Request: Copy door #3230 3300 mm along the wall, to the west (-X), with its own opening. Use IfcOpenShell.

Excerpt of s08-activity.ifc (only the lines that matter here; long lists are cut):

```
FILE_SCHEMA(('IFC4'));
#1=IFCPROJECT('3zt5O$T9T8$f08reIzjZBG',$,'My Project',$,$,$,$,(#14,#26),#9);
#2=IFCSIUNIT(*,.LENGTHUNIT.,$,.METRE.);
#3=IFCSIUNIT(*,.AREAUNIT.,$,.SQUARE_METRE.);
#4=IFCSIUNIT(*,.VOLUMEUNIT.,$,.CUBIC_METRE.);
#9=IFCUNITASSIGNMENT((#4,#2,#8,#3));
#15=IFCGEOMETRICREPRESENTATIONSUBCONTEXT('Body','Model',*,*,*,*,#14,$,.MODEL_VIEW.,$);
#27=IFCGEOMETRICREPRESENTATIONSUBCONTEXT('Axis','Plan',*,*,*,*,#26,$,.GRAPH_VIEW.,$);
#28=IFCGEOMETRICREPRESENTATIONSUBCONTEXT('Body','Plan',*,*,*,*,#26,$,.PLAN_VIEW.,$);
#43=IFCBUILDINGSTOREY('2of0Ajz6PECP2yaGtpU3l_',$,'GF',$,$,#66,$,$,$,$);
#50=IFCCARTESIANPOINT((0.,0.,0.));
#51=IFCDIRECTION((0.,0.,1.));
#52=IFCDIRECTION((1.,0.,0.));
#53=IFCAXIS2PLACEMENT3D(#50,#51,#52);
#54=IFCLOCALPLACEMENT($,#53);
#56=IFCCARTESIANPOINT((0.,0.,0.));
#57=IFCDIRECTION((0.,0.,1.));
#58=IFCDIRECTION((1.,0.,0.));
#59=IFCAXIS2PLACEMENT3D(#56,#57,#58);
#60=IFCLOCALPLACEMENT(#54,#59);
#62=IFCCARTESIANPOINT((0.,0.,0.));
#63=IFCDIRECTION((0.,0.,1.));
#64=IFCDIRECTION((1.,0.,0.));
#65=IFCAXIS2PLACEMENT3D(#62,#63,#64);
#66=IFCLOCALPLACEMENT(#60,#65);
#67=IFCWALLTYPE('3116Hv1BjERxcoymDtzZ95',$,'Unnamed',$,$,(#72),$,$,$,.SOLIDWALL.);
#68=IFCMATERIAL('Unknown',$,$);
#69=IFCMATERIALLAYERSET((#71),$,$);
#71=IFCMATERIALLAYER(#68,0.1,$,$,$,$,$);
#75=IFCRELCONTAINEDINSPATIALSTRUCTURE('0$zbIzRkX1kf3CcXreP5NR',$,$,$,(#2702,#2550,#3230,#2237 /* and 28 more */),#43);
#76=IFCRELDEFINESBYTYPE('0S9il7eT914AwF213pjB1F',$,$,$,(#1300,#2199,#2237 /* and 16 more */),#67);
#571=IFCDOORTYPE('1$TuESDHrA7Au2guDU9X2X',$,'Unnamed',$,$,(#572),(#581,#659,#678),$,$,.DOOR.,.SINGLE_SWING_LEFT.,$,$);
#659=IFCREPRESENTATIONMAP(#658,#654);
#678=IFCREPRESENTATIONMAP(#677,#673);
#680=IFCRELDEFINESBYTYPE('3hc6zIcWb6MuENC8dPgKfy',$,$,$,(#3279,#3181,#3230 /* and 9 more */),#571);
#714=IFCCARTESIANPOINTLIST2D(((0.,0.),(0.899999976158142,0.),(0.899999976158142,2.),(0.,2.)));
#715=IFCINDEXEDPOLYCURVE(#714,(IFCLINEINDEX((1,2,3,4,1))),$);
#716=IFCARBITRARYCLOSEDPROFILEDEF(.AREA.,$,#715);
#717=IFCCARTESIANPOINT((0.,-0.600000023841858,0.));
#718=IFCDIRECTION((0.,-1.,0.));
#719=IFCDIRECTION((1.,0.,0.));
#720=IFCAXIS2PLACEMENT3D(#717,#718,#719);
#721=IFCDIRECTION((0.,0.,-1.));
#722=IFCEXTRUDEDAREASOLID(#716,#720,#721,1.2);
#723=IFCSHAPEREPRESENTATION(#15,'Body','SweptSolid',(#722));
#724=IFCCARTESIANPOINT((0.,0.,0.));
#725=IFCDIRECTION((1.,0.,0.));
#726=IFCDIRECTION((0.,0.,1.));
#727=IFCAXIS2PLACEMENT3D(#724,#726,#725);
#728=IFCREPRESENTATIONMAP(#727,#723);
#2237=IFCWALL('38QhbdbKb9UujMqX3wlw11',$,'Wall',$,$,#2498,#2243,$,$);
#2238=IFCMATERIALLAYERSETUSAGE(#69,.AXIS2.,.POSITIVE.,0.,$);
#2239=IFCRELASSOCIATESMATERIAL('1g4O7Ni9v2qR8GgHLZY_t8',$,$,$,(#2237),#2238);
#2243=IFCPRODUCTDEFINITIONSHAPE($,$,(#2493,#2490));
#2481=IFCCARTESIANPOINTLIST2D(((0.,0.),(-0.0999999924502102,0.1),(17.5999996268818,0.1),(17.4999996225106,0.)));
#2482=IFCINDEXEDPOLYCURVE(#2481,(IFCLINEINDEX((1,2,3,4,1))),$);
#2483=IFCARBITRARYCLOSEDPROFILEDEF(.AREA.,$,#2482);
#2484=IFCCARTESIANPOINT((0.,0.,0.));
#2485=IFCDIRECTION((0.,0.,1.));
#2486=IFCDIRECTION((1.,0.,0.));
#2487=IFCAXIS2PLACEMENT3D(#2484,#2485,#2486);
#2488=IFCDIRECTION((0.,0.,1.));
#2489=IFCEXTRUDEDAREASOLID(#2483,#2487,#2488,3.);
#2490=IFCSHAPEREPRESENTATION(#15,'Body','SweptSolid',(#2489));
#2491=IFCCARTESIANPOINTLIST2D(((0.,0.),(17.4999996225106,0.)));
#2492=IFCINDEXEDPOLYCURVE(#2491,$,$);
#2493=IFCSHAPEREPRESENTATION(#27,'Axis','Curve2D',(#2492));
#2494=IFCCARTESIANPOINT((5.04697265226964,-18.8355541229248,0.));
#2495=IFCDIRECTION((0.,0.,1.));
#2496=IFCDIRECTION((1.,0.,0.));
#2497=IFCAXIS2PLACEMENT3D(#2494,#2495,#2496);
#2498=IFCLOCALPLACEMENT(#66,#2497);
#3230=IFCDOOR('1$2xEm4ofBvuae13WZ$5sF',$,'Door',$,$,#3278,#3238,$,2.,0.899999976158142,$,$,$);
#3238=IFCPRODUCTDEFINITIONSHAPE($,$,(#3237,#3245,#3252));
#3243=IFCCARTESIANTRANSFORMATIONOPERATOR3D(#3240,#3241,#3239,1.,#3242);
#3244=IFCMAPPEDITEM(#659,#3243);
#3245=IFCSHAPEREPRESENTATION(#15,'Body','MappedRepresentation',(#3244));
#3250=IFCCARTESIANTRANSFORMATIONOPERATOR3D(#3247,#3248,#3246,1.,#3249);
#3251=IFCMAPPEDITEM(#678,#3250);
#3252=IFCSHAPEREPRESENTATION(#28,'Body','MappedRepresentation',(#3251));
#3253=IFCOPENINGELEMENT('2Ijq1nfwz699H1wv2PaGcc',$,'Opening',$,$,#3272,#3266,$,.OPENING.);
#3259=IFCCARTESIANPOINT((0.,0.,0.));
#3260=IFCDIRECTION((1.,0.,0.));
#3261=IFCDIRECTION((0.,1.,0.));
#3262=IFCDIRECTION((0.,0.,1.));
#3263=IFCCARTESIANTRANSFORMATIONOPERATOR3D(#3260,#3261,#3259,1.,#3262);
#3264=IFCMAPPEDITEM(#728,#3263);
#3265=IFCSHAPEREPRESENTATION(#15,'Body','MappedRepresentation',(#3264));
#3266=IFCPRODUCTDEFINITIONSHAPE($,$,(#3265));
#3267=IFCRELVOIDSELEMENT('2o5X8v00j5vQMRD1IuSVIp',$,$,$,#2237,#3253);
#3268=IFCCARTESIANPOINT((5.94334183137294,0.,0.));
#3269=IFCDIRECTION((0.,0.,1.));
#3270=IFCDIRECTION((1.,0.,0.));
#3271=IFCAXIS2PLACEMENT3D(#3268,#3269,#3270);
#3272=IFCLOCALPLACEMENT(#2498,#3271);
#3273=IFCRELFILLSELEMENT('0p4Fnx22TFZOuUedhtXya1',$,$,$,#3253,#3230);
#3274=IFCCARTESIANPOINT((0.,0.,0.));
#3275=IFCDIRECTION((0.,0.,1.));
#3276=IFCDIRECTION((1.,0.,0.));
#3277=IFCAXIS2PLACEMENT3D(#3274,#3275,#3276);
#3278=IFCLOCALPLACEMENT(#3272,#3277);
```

```python
import ifcopenshell
import ifcopenshell.api.feature
import ifcopenshell.api.geometry
import ifcopenshell.api.root
import ifcopenshell.geom
import ifcopenshell.util.element
import ifcopenshell.util.placement
import ifcopenshell.util.shape
import ifcopenshell.util.unit

model = ifcopenshell.open("s08-activity.ifc")
unit_scale = ifcopenshell.util.unit.calculate_unit_scale(model)
settings = ifcopenshell.geom.settings()


def volume(element):
    """Net volume in cubic metres, openings subtracted."""
    shape = ifcopenshell.geom.create_shape(settings, element)
    return ifcopenshell.util.shape.get_volume(shape.geometry)


door = model.by_guid("1$2xEm4ofBvuae13WZ$5sF")
opening = door.FillsVoids[0].RelatingOpeningElement
wall = opening.VoidsElements[0].RelatingBuildingElement
before = volume(wall)
shift = ifcopenshell.util.placement.get_local_placement(wall.ObjectPlacement)[:3, 0] * -3.3 / unit_scale

# copy_class copies the void relationship, type, container and properties, but no geometry.
new_opening = ifcopenshell.api.root.copy_class(model, product=opening)
new_opening.Representation = ifcopenshell.util.element.copy_deep(
    model, opening.Representation, exclude=["IfcGeometricRepresentationContext", "IfcRepresentationMap"]
)
new_door = ifcopenshell.api.root.copy_class(model, product=door)
new_door.Representation = ifcopenshell.util.element.copy_deep(
    model, door.Representation, exclude=["IfcGeometricRepresentationContext", "IfcRepresentationMap"]
)
ifcopenshell.api.feature.add_filling(model, opening=new_opening, element=new_door)

for old, new in ((opening, new_opening), (door, new_door)):
    matrix = ifcopenshell.util.placement.get_local_placement(old.ObjectPlacement)
    matrix[:3, 3] += shift
    ifcopenshell.api.geometry.edit_object_placement(model, product=new, matrix=matrix, is_si=False)

after = volume(wall)

print(f"wall volume {before:.3f} -> {after:.3f} m3")

model.write("s08-activity_rev.ifc")
```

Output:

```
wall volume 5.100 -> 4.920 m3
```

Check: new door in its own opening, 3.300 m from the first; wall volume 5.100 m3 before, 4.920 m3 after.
